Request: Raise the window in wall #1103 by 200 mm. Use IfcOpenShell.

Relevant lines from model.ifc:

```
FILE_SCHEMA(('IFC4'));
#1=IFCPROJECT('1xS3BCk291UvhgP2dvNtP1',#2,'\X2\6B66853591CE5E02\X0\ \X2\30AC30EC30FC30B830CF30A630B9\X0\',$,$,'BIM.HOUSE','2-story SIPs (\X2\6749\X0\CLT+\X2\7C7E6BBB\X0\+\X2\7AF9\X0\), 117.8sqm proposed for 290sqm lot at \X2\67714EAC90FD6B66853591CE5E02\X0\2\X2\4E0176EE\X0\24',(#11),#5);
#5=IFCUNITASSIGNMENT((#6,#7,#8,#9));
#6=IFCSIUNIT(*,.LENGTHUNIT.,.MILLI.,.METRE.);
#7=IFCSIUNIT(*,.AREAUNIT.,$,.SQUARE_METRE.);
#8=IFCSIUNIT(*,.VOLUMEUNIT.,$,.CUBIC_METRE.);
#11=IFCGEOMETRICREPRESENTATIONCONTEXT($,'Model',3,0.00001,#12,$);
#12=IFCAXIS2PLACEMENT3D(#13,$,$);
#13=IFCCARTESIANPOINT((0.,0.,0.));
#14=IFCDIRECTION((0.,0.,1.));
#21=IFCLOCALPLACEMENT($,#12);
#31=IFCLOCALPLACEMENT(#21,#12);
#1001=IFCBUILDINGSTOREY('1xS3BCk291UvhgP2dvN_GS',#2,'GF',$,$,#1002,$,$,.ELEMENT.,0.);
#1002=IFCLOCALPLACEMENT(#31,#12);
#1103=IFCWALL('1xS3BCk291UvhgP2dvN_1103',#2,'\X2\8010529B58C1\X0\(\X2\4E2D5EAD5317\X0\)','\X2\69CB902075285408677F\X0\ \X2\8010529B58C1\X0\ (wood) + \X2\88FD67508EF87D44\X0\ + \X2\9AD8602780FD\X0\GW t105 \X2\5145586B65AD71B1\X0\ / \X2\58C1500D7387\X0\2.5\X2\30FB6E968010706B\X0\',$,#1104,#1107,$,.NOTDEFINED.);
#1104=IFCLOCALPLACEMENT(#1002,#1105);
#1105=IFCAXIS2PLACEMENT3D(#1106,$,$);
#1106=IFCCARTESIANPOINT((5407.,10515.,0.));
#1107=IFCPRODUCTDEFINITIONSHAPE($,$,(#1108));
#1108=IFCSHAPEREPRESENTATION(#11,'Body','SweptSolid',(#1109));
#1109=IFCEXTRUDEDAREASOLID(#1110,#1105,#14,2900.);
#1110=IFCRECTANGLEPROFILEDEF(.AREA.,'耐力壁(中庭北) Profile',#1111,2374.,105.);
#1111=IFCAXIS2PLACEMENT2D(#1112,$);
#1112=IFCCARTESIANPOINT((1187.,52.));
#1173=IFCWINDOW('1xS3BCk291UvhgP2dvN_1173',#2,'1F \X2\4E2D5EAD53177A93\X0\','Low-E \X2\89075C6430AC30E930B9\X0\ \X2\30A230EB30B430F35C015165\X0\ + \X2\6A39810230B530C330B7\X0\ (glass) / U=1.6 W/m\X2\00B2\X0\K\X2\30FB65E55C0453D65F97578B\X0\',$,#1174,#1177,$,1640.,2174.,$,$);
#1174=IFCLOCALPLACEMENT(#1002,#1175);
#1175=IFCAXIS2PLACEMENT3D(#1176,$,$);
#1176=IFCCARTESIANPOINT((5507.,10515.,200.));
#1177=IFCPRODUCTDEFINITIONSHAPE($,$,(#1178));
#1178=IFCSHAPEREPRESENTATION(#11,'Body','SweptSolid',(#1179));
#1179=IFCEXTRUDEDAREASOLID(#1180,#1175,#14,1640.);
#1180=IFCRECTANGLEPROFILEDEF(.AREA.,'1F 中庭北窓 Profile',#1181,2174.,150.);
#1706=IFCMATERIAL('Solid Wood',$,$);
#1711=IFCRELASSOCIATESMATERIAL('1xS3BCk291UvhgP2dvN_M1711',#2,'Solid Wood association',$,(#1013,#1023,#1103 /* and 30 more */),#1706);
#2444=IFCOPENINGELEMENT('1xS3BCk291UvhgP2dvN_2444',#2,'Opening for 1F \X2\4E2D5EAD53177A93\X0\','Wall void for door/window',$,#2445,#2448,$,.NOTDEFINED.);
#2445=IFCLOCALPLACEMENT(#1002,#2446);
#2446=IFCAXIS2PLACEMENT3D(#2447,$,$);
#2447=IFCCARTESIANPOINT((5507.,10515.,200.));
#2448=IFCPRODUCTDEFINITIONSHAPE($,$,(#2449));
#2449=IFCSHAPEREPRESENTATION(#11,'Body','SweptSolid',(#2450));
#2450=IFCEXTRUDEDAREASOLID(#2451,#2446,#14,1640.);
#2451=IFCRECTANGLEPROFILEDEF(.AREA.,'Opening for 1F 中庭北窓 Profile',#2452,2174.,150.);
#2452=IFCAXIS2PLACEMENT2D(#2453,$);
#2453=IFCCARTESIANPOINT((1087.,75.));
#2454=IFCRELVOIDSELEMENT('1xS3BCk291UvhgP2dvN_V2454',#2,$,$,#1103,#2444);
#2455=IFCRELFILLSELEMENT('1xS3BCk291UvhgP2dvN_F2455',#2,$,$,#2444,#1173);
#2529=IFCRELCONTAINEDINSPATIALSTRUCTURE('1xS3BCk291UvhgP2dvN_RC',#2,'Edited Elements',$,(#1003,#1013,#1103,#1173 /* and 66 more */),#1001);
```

```python
import numpy as np
import ifcopenshell
import ifcopenshell.api.geometry
import ifcopenshell.util.placement
import ifcopenshell.util.unit

model = ifcopenshell.open("model.ifc")
unit_scale = ifcopenshell.util.unit.calculate_unit_scale(model)

window = model.by_guid("1xS3BCk291UvhgP2dvN_1173")
opening = window.FillsVoids[0].RelatingOpeningElement
dz = 0.2 / unit_scale

shift = np.array([0.0, 0.0, dz])
# The window is not placed relative to its opening, so move both.
for product in (opening, window):
    matrix = ifcopenshell.util.placement.get_local_placement(product.ObjectPlacement)
    matrix[:3, 3] += shift
    ifcopenshell.api.geometry.edit_object_placement(model, product=product, matrix=matrix, is_si=False)

print(f"moved by {dz * unit_scale:+.3f} m")

model.write("model_edited.ifc")
```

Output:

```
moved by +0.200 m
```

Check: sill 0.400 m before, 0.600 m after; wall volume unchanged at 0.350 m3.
